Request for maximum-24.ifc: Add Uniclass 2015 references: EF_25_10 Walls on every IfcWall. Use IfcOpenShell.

First a look at what the model holds.

```python
import ifcopenshell

model = ifcopenshell.open("maximum-24.ifc")
print(model.schema)
print("classifications:", [c.Name for c in model.by_type("IfcClassification")])
for ifc_class in ("IfcDoor", "IfcRoof", "IfcStair", "IfcWall", "IfcWindow"):
    print(ifc_class, len(model.by_type(ifc_class)))
```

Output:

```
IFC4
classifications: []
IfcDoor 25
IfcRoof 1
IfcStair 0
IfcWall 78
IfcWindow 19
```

```python
import ifcopenshell
import ifcopenshell.api.classification

model = ifcopenshell.open("maximum-24.ifc")

system = ifcopenshell.api.classification.add_classification(model, classification="Uniclass 2015")

codes = {
    "IfcWall": ("EF_25_10", "Walls"),
}
for ifc_class, (code, name) in codes.items():
    products = model.by_type(ifc_class)
    ifcopenshell.api.classification.add_reference(
        model, products=products, classification=system, identification=code, name=name
    )
    print(code, len(products))

model.write("maximum-24_updated.ifc")
```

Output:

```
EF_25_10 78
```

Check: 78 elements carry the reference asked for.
